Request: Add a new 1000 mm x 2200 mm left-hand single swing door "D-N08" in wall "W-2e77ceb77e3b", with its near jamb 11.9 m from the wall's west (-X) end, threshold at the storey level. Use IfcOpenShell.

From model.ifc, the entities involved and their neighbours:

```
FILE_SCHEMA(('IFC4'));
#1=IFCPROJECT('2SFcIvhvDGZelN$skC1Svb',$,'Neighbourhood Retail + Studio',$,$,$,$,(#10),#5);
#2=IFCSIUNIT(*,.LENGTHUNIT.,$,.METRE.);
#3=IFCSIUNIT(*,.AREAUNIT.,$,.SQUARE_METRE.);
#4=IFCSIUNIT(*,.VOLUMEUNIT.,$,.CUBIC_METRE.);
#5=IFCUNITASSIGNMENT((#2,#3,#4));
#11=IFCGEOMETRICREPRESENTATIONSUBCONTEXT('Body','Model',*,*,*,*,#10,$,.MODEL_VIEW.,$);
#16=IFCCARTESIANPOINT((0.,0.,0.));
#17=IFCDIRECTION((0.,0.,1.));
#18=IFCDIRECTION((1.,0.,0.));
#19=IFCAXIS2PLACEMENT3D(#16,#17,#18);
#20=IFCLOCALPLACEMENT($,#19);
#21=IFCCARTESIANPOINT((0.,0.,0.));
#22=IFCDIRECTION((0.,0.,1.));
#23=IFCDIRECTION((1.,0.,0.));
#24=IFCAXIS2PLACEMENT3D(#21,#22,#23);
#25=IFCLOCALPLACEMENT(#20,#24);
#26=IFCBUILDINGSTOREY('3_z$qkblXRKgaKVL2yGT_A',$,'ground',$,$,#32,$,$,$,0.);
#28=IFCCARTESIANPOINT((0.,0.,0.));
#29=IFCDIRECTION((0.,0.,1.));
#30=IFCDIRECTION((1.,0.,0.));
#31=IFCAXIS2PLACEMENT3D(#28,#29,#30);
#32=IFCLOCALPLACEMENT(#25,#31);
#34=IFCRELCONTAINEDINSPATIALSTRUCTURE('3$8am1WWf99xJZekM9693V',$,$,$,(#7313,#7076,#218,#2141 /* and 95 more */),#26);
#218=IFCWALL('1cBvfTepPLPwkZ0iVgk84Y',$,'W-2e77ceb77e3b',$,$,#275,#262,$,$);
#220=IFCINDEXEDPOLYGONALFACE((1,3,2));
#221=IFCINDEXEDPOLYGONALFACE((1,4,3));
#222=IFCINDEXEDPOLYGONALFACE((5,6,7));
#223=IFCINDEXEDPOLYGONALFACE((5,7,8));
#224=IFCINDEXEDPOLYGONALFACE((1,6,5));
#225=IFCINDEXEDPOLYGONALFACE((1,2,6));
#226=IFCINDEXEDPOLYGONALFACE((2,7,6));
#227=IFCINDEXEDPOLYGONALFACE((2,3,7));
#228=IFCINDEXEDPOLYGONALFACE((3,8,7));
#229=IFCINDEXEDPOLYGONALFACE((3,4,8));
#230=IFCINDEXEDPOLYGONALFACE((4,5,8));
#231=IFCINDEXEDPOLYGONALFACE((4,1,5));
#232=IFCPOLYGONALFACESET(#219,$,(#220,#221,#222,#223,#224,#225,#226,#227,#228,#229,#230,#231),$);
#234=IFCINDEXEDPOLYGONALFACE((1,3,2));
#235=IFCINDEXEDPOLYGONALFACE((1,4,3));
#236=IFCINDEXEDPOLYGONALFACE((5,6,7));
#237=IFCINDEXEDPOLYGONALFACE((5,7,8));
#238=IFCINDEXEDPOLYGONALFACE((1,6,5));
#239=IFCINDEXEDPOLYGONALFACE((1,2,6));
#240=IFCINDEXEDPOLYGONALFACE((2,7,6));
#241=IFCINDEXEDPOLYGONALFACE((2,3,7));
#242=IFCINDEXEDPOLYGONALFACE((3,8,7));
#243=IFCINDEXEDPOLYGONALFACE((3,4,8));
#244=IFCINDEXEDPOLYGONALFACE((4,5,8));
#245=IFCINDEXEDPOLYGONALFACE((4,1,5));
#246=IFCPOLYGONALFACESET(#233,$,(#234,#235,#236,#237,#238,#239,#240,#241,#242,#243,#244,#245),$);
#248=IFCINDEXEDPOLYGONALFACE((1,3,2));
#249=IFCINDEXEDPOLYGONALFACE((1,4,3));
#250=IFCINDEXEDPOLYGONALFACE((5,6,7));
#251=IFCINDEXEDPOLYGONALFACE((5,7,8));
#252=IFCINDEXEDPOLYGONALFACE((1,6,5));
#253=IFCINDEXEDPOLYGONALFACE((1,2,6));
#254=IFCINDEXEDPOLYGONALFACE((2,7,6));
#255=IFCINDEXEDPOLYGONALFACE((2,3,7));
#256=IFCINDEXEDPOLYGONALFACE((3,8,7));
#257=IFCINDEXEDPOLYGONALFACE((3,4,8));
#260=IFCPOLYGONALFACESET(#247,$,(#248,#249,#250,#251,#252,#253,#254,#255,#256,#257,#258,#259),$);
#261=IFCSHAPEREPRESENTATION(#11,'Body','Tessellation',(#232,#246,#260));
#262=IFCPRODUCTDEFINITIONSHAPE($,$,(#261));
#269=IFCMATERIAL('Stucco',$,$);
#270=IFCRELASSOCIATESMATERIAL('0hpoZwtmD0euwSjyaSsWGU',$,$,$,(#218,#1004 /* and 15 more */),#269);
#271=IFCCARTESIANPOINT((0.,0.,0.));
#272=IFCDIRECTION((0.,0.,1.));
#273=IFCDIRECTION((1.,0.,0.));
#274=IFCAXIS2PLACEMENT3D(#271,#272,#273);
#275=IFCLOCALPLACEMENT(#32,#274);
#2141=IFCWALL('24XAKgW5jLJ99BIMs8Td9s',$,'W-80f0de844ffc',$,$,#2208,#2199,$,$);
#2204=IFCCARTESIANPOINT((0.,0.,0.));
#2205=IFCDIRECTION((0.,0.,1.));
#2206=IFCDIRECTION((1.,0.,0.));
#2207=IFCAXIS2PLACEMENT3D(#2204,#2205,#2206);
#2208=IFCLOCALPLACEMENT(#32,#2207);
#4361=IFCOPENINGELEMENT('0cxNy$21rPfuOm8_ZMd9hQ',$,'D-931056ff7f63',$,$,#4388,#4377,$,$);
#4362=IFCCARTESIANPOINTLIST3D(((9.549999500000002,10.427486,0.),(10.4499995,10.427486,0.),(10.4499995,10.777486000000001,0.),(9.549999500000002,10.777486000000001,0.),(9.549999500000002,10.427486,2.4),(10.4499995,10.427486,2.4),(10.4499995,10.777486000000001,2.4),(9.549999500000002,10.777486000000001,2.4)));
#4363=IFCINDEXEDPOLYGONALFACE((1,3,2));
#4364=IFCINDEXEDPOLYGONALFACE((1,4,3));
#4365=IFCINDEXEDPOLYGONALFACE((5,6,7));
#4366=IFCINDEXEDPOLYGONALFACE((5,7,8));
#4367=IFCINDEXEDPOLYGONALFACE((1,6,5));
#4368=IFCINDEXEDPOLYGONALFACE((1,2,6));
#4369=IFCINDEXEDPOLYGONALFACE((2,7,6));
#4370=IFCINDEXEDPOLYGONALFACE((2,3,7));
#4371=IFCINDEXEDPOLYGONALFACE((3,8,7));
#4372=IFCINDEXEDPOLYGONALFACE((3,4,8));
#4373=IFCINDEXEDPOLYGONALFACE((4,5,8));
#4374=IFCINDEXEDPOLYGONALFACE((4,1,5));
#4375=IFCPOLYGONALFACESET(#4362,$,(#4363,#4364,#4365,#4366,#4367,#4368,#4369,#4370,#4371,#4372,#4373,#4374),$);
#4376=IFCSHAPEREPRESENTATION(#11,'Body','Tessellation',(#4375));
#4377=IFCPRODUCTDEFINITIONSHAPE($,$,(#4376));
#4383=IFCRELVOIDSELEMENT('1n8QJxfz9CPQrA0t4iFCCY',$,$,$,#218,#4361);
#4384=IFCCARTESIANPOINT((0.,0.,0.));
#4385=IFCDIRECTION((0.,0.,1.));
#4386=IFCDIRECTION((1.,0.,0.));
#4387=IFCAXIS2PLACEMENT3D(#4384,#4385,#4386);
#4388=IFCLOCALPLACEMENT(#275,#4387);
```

```python
import numpy as np
import ifcopenshell
import ifcopenshell.api.feature
import ifcopenshell.api.geometry
import ifcopenshell.api.root
import ifcopenshell.api.spatial
import ifcopenshell.geom
import ifcopenshell.util.element
import ifcopenshell.util.placement
import ifcopenshell.util.representation
import ifcopenshell.util.shape
import ifcopenshell.util.unit

model = ifcopenshell.open("model.ifc")
unit_scale = ifcopenshell.util.unit.calculate_unit_scale(model)
settings = ifcopenshell.geom.settings()


def volume(element):
    """Net volume in cubic metres, openings subtracted."""
    shape = ifcopenshell.geom.create_shape(settings, element)
    return ifcopenshell.util.shape.get_volume(shape.geometry)


wall = model.by_id(218)
storey = ifcopenshell.util.element.get_container(wall, ifc_class="IfcBuildingStorey")
context = ifcopenshell.util.representation.get_context(model, "Model", "Body", "MODEL_VIEW")
before = volume(wall)

width, height, from_end, sill = 1, 2.2, 11.9, 0.0  # metres

# The wall runs along its own X axis, and the end named is its -X end.
wall_shape = ifcopenshell.geom.create_shape(settings, wall)
x, y, z = ifcopenshell.util.shape.get_vertices(wall_shape.geometry).T
start = x.min() + from_end
face, thickness = float(y.min()), float(y.max() - y.min())
wall_matrix = ifcopenshell.util.placement.get_local_placement(wall.ObjectPlacement)
level = ifcopenshell.util.placement.get_local_placement(storey.ObjectPlacement)[2, 3]


def in_wall(x, y):
    """Placement at x, y metres in the wall's axes, at sill height."""
    matrix = wall_matrix.copy()
    matrix[:, 3] = wall_matrix @ np.array([x / unit_scale, y / unit_scale, 0.0, 1.0])
    matrix[2, 3] = level + sill / unit_scale
    return matrix


# Opening: a box that overshoots both wall faces by 50 mm.
opening = ifcopenshell.api.root.create_entity(model, ifc_class="IfcOpeningElement", predefined_type="OPENING")
box = ifcopenshell.api.geometry.add_wall_representation(
    model, context=context, length=width, height=height, thickness=thickness + 0.1
)
ifcopenshell.api.geometry.assign_representation(model, product=opening, representation=box)
ifcopenshell.api.geometry.edit_object_placement(model, product=opening, matrix=in_wall(start, face - 0.05), is_si=False)
ifcopenshell.api.feature.add_feature(model, feature=opening, element=wall)

door = ifcopenshell.api.root.create_entity(model, ifc_class="IfcDoor", name="D-N08", predefined_type="DOOR")
door.OverallWidth, door.OverallHeight = width / unit_scale, height / unit_scale
door.OperationType = "SINGLE_SWING_LEFT"
body = ifcopenshell.api.geometry.add_door_representation(
    model,
    context=context,
    overall_width=door.OverallWidth,
    overall_height=door.OverallHeight,
    operation_type="SINGLE_SWING_LEFT",
    lining_properties={"LiningDepth": thickness / unit_scale, "ThresholdDepth": thickness / unit_scale},
)
ifcopenshell.api.geometry.assign_representation(model, product=door, representation=body)
ifcopenshell.api.spatial.assign_container(model, products=[door], relating_structure=storey)
ifcopenshell.api.feature.add_filling(model, opening=opening, element=door)

# The lining spans the wall, so the door starts at the wall face.
ifcopenshell.api.geometry.edit_object_placement(model, product=door, matrix=in_wall(start, face), is_si=False)

after = volume(wall)

print(f"wall volume {before:.3f} -> {after:.3f} m3")

model.write("model_updated.ifc")
```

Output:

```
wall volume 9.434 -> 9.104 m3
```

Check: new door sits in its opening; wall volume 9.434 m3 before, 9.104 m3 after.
